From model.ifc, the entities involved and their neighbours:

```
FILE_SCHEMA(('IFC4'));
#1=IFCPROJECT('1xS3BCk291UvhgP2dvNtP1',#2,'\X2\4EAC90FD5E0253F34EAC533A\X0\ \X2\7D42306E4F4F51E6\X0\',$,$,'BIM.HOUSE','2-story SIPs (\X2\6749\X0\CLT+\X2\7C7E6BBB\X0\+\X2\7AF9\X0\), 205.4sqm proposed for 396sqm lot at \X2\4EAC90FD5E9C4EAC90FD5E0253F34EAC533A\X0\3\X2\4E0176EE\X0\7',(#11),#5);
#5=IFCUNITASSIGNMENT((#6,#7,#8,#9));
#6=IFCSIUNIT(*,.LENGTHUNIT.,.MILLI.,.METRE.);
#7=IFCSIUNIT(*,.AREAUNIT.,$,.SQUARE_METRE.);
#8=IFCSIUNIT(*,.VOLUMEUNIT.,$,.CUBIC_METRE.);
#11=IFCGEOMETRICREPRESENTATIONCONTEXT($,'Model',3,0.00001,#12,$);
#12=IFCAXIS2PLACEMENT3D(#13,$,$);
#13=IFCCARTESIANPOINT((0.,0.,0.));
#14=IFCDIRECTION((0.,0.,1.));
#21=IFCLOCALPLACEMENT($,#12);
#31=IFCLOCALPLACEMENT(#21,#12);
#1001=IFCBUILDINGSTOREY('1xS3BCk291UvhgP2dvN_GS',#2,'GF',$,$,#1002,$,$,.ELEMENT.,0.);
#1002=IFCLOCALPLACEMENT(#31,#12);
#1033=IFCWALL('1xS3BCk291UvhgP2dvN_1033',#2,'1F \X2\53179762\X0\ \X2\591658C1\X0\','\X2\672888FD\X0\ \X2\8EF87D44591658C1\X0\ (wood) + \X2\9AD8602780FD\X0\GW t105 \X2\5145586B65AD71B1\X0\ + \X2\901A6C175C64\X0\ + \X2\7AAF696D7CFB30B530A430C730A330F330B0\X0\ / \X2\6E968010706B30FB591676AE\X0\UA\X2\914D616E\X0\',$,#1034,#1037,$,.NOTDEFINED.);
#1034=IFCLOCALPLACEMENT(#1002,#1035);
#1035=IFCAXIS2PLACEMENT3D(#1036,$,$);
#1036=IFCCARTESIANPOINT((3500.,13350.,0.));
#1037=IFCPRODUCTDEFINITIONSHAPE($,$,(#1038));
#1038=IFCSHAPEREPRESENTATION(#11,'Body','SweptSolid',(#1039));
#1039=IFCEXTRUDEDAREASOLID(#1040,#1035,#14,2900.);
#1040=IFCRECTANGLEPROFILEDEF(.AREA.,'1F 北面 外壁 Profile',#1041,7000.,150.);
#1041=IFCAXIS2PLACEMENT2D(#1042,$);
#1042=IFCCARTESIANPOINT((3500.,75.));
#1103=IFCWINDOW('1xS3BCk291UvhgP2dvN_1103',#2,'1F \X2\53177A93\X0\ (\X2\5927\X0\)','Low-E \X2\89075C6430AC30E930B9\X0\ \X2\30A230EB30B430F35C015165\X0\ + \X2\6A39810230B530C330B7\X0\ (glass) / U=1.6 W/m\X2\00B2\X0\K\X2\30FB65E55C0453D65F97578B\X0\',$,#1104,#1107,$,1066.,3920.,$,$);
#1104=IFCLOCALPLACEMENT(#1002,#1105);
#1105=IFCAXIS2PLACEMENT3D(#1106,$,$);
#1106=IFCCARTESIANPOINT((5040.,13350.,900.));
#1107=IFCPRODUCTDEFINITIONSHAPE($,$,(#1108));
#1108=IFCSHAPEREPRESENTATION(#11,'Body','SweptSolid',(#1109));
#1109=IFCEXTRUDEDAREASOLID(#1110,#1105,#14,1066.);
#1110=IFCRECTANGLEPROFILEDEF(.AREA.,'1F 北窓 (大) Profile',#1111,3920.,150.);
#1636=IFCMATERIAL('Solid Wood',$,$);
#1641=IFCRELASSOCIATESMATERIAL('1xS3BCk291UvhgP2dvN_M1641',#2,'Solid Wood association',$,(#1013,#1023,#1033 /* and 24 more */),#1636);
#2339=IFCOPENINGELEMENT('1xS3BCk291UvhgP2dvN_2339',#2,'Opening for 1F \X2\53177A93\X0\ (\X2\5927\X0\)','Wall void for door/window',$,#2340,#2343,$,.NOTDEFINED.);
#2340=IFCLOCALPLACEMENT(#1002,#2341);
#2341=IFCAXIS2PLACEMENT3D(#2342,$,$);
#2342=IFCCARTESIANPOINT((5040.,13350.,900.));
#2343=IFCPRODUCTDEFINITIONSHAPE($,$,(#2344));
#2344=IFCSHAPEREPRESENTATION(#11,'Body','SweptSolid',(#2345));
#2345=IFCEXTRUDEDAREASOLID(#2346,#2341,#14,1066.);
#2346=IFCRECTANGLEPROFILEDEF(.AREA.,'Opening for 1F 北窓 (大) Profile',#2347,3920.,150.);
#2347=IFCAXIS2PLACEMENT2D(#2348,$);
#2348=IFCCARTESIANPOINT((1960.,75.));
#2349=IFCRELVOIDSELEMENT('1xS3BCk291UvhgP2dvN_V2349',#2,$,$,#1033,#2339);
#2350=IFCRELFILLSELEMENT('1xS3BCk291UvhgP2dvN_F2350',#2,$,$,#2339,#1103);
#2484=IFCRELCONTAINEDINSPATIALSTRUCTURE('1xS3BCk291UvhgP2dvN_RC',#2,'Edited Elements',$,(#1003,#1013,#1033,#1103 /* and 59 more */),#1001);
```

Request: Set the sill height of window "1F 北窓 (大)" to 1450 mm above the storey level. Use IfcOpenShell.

```python
import numpy as np
import ifcopenshell
import ifcopenshell.api.geometry
import ifcopenshell.geom
import ifcopenshell.util.element
import ifcopenshell.util.placement
import ifcopenshell.util.shape
import ifcopenshell.util.unit

model = ifcopenshell.open("model.ifc")
unit_scale = ifcopenshell.util.unit.calculate_unit_scale(model)

window = model.by_guid("1xS3BCk291UvhgP2dvN_1103")
opening = window.FillsVoids[0].RelatingOpeningElement
storey = ifcopenshell.util.element.get_container(window, ifc_class="IfcBuildingStorey")
level = ifcopenshell.util.placement.get_local_placement(storey.ObjectPlacement)[2, 3]

# The opening's origin need not be at the sill, so measure its lowest point.
shape = ifcopenshell.geom.create_shape(ifcopenshell.geom.settings(), opening)
bottom = ifcopenshell.util.shape.get_shape_bottom_elevation(shape, shape.geometry) / unit_scale
dz = level + 1.45 / unit_scale - bottom

shift = np.array([0.0, 0.0, dz])
# The window is not placed relative to its opening, so move both.
for product in (opening, window):
    matrix = ifcopenshell.util.placement.get_local_placement(product.ObjectPlacement)
    matrix[:3, 3] += shift
    ifcopenshell.api.geometry.edit_object_placement(model, product=product, matrix=matrix, is_si=False)

print(f"moved by {dz * unit_scale:+.3f} m")

model.write("model-out.ifc")
```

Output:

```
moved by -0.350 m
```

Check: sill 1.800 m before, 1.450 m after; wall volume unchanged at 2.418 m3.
